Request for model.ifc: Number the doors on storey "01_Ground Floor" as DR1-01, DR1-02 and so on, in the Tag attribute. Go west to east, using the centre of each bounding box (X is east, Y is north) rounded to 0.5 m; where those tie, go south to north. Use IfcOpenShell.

First a look at what the model holds.

```python
import ifcopenshell
import ifcopenshell.util.element
import ifcopenshell.util.placement

model = ifcopenshell.open("model.ifc")
print(model.schema)
storey = next(s for s in model.by_type("IfcBuildingStorey") if s.Name == "01_Ground Floor")
doors = [e for e in ifcopenshell.util.element.get_decomposition(storey) if e.is_a("IfcDoor")]
for e in sorted(doors, key=lambda e: e.id()):
    origin = ifcopenshell.util.placement.get_local_placement(e.ObjectPlacement)[:3, 3]
    print(e.id(), e.Tag, e.Name, origin.round(2) + 0.0, sep=" | ")
```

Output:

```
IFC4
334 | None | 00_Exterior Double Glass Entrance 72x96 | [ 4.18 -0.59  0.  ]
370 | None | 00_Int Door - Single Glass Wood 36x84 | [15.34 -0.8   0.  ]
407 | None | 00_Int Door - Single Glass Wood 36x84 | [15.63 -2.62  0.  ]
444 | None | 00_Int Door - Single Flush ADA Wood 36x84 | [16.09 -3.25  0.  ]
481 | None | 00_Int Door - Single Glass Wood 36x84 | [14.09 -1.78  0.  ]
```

```python
import ifcopenshell
import ifcopenshell.geom
import ifcopenshell.util.element
import ifcopenshell.util.shape

model = ifcopenshell.open("model.ifc")
settings = ifcopenshell.geom.settings()
settings.set("use-world-coords", True)


def centre(element):
    shape = ifcopenshell.geom.create_shape(settings, element)
    return ifcopenshell.util.shape.get_bbox_centroid(shape.geometry)


storey = next(s for s in model.by_type("IfcBuildingStorey") if s.Name == "01_Ground Floor")
doors = [e for e in ifcopenshell.util.element.get_decomposition(storey) if e.is_a("IfcDoor")]

# Insertion points can sit at a corner or the storey origin, so sort by the geometry (in metres).
centres = {e: centre(e) for e in doors}
doors.sort(key=lambda e: (round(centres[e][0] / 0.5), centres[e][1]))

for i, e in enumerate(doors, start=1):
    number = f"DR1-{i:02d}"
    e.Tag = number
    print(e.id(), number)

model.write("model_rev.ifc")
```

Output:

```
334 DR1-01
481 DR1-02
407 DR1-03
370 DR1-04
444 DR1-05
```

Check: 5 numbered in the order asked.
